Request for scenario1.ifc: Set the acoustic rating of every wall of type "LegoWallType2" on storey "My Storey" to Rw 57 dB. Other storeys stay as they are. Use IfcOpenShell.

First a look at what the model holds.

```python
import ifcopenshell
import ifcopenshell.util.element

model = ifcopenshell.open("scenario1.ifc")
print(model.schema)
storey = next(s for s in model.by_type("IfcBuildingStorey") if s.Name == "My Storey")
walls = [e for e in ifcopenshell.util.element.get_decomposition(storey) if e.is_a("IfcWall")]
seen = {}
for e in walls:
    element_type = ifcopenshell.util.element.get_type(e)
    key = (element_type.Name if element_type != e and element_type else None, ifcopenshell.util.element.get_pset(e, "Pset_WallCommon", "AcousticRating"))
    seen[key] = seen.get(key, 0) + 1
for (name, value), count in sorted(seen.items(), key=str):
    print(count, "x", name, "|", value)
```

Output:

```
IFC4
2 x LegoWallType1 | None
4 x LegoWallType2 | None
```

```python
import ifcopenshell
import ifcopenshell.api.pset
import ifcopenshell.util.element

model = ifcopenshell.open("scenario1.ifc")

storey = next(s for s in model.by_type("IfcBuildingStorey") if s.Name == "My Storey")
walls = [e for e in ifcopenshell.util.element.get_decomposition(storey) if e.is_a("IfcWall")]

count = 0
for e in walls:
    element_type = ifcopenshell.util.element.get_type(e)
    if element_type in (None, e) or element_type.Name != "LegoWallType2":
        continue
    # add_pset returns the element's existing set when there is one.
    pset = ifcopenshell.api.pset.add_pset(model, product=e, name="Pset_WallCommon")
    ifcopenshell.api.pset.edit_pset(model, pset=pset, properties={"AcousticRating": "Rw 57 dB"})
    count += 1

print(count, "walls updated")

model.write("scenario1-out.ifc")
```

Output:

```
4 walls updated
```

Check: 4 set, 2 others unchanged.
